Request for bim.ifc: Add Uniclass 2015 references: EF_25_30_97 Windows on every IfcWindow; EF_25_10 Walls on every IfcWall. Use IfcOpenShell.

First a look at what the model holds.

```python
import ifcopenshell

model = ifcopenshell.open("bim.ifc")
print(model.schema)
print("classifications:", [c.Name for c in model.by_type("IfcClassification")])
for ifc_class in ("IfcDoor", "IfcRoof", "IfcStair", "IfcWall", "IfcWindow"):
    print(ifc_class, len(model.by_type(ifc_class)))
```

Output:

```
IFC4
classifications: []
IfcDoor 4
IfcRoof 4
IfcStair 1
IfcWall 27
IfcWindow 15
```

```python
import ifcopenshell
import ifcopenshell.api.classification

model = ifcopenshell.open("bim.ifc")

system = ifcopenshell.api.classification.add_classification(model, classification="Uniclass 2015")

codes = {
    "IfcWindow": ("EF_25_30_97", "Windows"),
    "IfcWall": ("EF_25_10", "Walls"),
}
for ifc_class, (code, name) in codes.items():
    products = model.by_type(ifc_class)
    ifcopenshell.api.classification.add_reference(
        model, products=products, classification=system, identification=code, name=name
    )
    print(code, len(products))

model.write("bim_v2.ifc")
```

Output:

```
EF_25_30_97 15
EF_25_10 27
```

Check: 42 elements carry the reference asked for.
